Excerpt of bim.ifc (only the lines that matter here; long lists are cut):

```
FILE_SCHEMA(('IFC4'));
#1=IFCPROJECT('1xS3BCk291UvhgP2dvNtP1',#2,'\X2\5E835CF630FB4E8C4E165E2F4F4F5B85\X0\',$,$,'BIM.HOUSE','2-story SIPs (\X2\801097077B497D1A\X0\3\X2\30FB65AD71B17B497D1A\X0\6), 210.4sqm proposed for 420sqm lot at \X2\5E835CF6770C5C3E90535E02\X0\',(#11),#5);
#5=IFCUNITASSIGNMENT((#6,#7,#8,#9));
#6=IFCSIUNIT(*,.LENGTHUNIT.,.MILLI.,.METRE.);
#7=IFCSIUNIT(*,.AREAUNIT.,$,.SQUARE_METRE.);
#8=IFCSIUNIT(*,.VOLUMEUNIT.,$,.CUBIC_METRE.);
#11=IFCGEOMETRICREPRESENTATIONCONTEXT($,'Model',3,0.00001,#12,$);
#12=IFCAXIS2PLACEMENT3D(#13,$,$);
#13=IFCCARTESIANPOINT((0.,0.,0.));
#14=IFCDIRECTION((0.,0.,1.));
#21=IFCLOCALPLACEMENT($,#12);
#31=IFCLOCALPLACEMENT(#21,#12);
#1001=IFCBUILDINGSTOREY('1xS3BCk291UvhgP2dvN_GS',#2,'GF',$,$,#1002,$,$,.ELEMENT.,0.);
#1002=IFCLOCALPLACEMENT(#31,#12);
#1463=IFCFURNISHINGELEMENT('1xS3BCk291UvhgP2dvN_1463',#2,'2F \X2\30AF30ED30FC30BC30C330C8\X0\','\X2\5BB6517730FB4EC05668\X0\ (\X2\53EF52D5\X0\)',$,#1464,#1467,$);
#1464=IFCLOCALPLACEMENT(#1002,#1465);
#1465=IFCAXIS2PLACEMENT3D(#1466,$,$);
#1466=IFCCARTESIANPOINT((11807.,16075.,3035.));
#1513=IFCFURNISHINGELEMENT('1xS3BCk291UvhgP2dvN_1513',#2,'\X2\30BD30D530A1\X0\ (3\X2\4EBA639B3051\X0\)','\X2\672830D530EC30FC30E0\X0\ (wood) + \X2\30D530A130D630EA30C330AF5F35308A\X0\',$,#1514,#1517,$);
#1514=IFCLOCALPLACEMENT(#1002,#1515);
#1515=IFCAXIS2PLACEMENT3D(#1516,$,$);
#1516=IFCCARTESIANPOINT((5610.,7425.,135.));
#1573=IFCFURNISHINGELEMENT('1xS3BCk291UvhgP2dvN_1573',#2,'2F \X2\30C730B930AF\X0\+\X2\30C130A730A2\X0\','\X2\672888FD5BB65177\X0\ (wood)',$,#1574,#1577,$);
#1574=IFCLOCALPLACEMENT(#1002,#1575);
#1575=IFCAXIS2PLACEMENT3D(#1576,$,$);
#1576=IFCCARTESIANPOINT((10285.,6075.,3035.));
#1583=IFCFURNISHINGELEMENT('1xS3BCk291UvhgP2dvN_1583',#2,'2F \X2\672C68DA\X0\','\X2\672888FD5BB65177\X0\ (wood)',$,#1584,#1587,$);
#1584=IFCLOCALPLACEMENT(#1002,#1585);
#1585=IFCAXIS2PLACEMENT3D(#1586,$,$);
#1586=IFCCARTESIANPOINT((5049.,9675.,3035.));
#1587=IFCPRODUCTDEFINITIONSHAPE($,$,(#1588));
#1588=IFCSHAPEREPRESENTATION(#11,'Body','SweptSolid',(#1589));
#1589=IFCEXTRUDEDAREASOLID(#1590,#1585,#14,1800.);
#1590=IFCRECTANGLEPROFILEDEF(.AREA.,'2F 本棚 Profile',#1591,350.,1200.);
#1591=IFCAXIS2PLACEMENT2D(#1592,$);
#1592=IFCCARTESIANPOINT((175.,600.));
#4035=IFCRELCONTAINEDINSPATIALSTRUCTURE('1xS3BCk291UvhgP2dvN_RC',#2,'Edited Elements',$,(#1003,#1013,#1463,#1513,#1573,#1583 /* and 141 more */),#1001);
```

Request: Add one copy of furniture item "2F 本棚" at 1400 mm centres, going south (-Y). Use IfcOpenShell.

```python
import numpy as np
import ifcopenshell
import ifcopenshell.api.geometry
import ifcopenshell.api.root
import ifcopenshell.util.element
import ifcopenshell.util.placement

model = ifcopenshell.open("bim.ifc")


def reuse_history(source, copy):
    """copy_class also copies each property set's owner history, people and application; keep the originals."""
    for rel in copy.IsDefinedBy:
        if rel.is_a("IfcRelDefinesByProperties") and (history := rel.RelatingPropertyDefinition.OwnerHistory):
            rel.RelatingPropertyDefinition.OwnerHistory = source.OwnerHistory
            ifcopenshell.util.element.remove_deep2(model, history)


source = model.by_id(1583)
base = ifcopenshell.util.placement.get_local_placement(source.ObjectPlacement)
step = np.array([0.0, -1.0, 0.0]) * 1400.0

for i in range(1, 2):
    copy = ifcopenshell.api.root.copy_class(model, product=source)
    copy.Representation = ifcopenshell.util.element.copy_deep(
        model, source.Representation, exclude=["IfcGeometricRepresentationContext", "IfcRepresentationMap"]
    )
    reuse_history(source, copy)
    matrix = base.copy()
    matrix[:3, 3] += i * step
    print("added at", matrix[:3, 3].round(3) + 0.0)
    ifcopenshell.api.geometry.edit_object_placement(model, product=copy, matrix=matrix, is_si=False)

model.write("bim-out.ifc")
```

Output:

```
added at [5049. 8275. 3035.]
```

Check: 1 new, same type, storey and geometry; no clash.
